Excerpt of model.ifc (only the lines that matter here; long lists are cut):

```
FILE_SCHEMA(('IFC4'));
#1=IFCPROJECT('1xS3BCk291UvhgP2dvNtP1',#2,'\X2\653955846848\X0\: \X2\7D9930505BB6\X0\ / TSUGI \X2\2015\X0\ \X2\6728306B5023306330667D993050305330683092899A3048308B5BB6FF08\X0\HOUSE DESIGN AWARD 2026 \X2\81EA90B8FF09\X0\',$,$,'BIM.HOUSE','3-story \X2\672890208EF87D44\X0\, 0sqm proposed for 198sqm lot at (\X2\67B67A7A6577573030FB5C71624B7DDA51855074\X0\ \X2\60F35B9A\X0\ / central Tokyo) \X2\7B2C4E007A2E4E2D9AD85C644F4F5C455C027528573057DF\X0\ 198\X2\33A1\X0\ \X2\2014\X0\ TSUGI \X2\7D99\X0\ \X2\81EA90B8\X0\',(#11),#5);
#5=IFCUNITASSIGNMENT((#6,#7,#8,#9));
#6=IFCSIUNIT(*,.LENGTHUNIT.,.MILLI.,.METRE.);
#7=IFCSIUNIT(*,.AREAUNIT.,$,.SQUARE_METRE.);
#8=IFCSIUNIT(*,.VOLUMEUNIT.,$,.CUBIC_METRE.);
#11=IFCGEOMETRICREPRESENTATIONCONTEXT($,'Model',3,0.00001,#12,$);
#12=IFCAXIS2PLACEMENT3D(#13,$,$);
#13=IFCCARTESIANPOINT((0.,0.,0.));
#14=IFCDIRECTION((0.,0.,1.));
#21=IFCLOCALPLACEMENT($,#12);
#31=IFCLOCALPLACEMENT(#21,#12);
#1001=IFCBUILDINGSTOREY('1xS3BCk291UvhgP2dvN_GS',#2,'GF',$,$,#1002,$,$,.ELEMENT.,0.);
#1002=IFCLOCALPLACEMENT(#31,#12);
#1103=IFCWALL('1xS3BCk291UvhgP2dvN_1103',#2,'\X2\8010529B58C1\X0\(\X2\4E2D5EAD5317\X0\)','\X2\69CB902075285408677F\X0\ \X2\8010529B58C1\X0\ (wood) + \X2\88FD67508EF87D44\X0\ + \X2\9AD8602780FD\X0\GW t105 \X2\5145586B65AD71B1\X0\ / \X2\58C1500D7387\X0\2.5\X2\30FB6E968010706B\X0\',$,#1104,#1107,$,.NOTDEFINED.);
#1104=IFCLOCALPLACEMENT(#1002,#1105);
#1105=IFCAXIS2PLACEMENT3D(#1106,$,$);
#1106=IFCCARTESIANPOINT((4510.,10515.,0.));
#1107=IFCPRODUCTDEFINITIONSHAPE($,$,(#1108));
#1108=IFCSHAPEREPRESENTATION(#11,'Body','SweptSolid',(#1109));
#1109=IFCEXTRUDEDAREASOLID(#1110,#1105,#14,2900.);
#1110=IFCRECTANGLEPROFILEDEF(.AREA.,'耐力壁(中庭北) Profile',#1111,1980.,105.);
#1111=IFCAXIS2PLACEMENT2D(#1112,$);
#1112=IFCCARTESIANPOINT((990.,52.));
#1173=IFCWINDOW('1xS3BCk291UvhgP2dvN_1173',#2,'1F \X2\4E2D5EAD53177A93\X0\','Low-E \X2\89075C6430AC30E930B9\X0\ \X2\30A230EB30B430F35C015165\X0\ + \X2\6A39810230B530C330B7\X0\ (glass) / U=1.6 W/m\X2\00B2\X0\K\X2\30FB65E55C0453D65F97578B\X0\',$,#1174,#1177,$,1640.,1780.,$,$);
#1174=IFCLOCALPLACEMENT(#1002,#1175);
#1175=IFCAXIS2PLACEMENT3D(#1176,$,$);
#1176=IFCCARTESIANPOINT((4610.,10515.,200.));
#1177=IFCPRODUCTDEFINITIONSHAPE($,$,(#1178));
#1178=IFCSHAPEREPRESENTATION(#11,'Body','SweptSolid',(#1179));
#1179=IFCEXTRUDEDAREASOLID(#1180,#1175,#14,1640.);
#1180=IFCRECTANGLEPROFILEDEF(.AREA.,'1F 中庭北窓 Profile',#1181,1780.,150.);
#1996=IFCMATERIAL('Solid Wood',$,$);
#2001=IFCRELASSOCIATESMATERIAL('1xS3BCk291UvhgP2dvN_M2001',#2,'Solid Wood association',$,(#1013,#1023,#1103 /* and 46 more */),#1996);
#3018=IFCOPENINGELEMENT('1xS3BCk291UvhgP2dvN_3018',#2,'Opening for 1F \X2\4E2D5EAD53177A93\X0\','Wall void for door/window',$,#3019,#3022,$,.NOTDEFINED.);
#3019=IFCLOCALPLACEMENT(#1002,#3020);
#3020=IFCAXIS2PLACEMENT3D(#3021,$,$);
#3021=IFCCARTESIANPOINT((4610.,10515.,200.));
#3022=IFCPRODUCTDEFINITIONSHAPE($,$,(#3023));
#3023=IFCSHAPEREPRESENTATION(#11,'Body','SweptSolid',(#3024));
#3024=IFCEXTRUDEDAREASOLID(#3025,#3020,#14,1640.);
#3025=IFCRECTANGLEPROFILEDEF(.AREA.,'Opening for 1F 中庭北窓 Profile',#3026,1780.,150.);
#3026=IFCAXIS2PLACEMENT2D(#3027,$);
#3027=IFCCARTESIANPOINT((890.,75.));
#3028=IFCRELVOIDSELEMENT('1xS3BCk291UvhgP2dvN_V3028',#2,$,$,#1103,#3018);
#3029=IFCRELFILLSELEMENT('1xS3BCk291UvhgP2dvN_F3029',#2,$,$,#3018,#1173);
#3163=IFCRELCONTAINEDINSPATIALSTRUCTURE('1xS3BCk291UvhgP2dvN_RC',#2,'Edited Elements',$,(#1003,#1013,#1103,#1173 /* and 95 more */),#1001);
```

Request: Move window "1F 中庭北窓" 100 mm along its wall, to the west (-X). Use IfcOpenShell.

```python
import ifcopenshell
import ifcopenshell.api.geometry
import ifcopenshell.util.placement

model = ifcopenshell.open("model.ifc")

window = model.by_id(1173)
opening = window.FillsVoids[0].RelatingOpeningElement
wall = opening.VoidsElements[0].RelatingBuildingElement

wall_matrix = ifcopenshell.util.placement.get_local_placement(wall.ObjectPlacement)
shift = wall_matrix[:3, 0] * -100.0
before = ifcopenshell.util.placement.get_local_placement(window.ObjectPlacement)[:3, 3].copy()

# The window is not placed relative to its opening, so move both.
for product in (opening, window):
    matrix = ifcopenshell.util.placement.get_local_placement(product.ObjectPlacement)
    matrix[:3, 3] += shift
    ifcopenshell.api.geometry.edit_object_placement(model, product=product, matrix=matrix, is_si=False)

after = ifcopenshell.util.placement.get_local_placement(window.ObjectPlacement)[:3, 3]
print("window moved by", (after - before).round(3) + 0.0)

model.write("model_updated.ifc")
```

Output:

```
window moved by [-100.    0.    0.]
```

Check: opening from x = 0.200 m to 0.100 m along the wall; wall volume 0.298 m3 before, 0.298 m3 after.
